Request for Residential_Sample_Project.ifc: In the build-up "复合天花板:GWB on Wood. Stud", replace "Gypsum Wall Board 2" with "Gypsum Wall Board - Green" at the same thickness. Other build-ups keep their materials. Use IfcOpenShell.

First a look at what the model holds.

```python
import ifcopenshell
import ifcopenshell.util.element

model = ifcopenshell.open("Residential_Sample_Project.ifc")
print(model.schema)
for layer_set in model.by_type("IfcMaterialLayerSet"):
    if layer_set.LayerSetName == "复合天花板:GWB on Wood. Stud":
        for layer in layer_set.MaterialLayers:
            print(layer.id(), layer.Material and layer.Material.Name, layer.LayerThickness, sep=" | ")
        print(len(ifcopenshell.util.element.get_elements_by_material(model, layer_set)), "elements and types use it")
print(sorted(m.Name for m in model.by_type("IfcMaterial") if m.Name)[:60])
```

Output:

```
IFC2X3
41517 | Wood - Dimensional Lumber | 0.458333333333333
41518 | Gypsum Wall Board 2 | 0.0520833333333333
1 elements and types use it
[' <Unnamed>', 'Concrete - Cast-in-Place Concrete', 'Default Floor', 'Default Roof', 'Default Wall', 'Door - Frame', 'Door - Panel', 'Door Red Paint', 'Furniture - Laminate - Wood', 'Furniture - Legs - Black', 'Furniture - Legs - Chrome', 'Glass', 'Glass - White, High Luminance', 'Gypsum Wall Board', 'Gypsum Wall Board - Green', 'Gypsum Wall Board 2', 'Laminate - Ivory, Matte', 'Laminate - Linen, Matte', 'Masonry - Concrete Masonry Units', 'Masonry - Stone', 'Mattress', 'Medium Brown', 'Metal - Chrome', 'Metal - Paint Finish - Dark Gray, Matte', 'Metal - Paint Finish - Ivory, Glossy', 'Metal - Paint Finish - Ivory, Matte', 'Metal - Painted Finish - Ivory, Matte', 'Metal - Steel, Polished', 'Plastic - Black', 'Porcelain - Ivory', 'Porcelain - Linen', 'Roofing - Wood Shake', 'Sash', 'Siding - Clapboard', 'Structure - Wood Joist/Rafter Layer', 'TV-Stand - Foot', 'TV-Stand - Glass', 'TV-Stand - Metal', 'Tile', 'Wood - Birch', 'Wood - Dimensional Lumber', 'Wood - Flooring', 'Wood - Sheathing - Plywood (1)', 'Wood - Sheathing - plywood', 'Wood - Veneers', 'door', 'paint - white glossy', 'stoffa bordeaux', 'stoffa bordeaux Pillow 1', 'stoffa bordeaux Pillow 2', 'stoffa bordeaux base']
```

```python
import ifcopenshell
import ifcopenshell.api.material

model = ifcopenshell.open("Residential_Sample_Project.ifc")

layer_set = next(s for s in model.by_type("IfcMaterialLayerSet") if s.LayerSetName == "复合天花板:GWB on Wood. Stud")
layer = next(l for l in layer_set.MaterialLayers if l.Material and l.Material.Name == "Gypsum Wall Board 2")
material = next(m for m in model.by_type("IfcMaterial") if m.Name == "Gypsum Wall Board - Green")

# Point this one layer at the other material; renaming the old one would change it everywhere.
ifcopenshell.api.material.edit_layer(model, layer=layer, attributes={}, material=material)

print([l.Material.Name if l.Material else None for l in layer_set.MaterialLayers])

model.write("Residential_Sample_Project_updated.ifc")
```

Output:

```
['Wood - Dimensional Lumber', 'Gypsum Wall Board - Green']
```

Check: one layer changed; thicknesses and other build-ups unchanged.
